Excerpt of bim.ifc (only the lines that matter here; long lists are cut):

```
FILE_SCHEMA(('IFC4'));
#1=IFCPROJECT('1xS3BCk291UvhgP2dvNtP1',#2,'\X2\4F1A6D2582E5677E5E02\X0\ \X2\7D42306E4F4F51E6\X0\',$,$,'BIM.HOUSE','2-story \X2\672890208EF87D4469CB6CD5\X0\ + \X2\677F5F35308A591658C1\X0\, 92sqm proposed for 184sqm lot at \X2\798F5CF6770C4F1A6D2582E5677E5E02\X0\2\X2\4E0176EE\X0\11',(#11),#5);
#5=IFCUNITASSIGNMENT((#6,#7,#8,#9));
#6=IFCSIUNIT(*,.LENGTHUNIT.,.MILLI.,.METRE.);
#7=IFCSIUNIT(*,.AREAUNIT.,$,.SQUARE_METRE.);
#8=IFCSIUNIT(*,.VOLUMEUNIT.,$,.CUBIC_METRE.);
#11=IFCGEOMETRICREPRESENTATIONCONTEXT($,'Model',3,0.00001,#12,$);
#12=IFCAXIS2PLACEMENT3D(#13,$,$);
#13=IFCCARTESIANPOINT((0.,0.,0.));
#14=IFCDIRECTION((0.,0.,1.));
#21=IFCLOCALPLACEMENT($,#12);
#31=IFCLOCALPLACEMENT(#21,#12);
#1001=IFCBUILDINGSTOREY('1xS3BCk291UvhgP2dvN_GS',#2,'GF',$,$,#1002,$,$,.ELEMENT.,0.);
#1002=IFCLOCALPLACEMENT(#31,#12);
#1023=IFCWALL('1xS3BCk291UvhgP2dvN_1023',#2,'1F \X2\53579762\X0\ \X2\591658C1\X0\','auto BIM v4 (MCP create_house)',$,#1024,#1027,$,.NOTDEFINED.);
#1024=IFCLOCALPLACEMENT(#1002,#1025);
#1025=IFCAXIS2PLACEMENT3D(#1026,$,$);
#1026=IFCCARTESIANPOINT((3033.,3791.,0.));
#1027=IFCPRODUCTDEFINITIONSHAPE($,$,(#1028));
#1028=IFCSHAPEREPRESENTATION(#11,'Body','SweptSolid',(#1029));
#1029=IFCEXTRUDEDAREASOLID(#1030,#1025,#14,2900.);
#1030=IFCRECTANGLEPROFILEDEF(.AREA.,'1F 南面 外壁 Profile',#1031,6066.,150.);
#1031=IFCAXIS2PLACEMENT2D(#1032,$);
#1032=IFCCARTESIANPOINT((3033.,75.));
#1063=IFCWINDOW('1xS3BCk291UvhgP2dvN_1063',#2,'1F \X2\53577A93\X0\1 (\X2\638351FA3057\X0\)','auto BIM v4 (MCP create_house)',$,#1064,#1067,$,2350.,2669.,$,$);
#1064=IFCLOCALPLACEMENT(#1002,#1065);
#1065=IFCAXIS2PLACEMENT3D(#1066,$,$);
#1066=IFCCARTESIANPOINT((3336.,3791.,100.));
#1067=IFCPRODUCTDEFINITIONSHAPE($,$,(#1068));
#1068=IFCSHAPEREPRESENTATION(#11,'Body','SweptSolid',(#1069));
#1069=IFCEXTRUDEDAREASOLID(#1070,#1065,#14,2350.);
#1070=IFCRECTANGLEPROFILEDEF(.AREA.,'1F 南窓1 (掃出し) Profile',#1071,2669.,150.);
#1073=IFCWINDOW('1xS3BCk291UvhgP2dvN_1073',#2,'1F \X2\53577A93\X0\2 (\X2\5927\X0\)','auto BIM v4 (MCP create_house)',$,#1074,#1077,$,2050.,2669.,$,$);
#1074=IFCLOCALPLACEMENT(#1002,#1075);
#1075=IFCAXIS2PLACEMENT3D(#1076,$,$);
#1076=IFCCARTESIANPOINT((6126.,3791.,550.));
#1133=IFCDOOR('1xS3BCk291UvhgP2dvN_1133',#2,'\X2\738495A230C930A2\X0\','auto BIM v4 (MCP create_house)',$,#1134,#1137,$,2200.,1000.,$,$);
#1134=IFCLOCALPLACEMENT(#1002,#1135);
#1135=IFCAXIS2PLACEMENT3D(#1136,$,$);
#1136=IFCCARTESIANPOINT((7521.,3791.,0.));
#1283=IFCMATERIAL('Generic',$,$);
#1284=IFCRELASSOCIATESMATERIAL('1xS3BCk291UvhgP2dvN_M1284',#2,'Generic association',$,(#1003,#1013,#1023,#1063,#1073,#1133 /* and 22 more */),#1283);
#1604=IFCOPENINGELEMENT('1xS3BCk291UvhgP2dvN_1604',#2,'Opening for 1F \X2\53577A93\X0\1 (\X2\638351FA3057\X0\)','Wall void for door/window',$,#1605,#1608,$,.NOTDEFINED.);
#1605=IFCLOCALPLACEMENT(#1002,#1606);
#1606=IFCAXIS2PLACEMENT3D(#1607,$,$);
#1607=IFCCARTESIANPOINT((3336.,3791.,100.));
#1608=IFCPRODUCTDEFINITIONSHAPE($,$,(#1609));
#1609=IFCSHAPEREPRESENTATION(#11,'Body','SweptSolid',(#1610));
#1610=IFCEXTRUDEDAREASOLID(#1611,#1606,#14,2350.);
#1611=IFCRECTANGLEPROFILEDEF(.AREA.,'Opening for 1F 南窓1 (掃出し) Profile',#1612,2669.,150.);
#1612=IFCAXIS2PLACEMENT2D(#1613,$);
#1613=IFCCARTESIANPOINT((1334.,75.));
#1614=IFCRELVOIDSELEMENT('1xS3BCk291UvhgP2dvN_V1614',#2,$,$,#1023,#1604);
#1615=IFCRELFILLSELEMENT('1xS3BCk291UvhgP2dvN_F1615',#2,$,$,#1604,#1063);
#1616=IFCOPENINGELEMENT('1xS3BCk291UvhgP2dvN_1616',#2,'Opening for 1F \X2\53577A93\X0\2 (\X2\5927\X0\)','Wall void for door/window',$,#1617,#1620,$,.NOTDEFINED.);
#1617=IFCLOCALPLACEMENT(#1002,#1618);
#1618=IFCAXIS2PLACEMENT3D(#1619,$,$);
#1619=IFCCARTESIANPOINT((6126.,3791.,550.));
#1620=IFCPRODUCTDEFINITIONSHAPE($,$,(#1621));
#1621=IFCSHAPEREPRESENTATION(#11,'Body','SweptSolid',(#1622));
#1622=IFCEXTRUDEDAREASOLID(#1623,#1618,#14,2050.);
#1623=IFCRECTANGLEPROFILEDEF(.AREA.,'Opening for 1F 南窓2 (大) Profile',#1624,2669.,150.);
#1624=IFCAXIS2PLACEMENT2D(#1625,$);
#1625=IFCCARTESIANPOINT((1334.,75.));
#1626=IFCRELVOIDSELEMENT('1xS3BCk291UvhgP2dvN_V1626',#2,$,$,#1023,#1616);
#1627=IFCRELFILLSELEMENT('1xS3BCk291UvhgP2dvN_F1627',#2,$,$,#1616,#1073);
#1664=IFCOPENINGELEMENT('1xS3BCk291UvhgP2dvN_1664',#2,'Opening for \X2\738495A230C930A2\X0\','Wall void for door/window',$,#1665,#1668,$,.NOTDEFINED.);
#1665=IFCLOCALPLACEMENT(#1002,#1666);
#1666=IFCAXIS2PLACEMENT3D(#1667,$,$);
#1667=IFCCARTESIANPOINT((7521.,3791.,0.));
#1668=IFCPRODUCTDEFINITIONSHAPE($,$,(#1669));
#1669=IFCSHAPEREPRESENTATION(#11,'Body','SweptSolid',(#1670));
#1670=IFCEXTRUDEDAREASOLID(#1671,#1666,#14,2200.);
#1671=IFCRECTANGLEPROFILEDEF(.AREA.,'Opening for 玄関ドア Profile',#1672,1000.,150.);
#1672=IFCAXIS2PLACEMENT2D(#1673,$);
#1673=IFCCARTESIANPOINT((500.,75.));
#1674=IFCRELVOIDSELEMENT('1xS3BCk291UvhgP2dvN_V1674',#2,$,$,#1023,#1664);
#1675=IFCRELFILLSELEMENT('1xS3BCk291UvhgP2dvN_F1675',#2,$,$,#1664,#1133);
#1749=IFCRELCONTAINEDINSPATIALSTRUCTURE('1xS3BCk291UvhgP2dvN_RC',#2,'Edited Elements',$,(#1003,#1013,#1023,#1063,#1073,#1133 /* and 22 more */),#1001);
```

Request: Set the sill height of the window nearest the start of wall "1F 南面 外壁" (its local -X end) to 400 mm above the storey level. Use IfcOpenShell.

```python
import numpy as np
import ifcopenshell
import ifcopenshell.api.geometry
import ifcopenshell.geom
import ifcopenshell.util.element
import ifcopenshell.util.placement
import ifcopenshell.util.shape
import ifcopenshell.util.unit

model = ifcopenshell.open("bim.ifc")
unit_scale = ifcopenshell.util.unit.calculate_unit_scale(model)

window = model.by_guid("1xS3BCk291UvhgP2dvN_1063")
opening = window.FillsVoids[0].RelatingOpeningElement
storey = ifcopenshell.util.element.get_container(window, ifc_class="IfcBuildingStorey")
level = ifcopenshell.util.placement.get_local_placement(storey.ObjectPlacement)[2, 3]

# The opening's origin need not be at the sill, so measure its lowest point.
shape = ifcopenshell.geom.create_shape(ifcopenshell.geom.settings(), opening)
bottom = ifcopenshell.util.shape.get_shape_bottom_elevation(shape, shape.geometry) / unit_scale
dz = level + 0.4 / unit_scale - bottom

shift = np.array([0.0, 0.0, dz])
# The window is not placed relative to its opening, so move both.
for product in (opening, window):
    matrix = ifcopenshell.util.placement.get_local_placement(product.ObjectPlacement)
    matrix[:3, 3] += shift
    ifcopenshell.api.geometry.edit_object_placement(model, product=product, matrix=matrix, is_si=False)

print(f"moved by {dz * unit_scale:+.3f} m")

model.write("bim_edited.ifc")
```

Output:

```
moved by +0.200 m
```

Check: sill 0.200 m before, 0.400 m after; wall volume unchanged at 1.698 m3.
